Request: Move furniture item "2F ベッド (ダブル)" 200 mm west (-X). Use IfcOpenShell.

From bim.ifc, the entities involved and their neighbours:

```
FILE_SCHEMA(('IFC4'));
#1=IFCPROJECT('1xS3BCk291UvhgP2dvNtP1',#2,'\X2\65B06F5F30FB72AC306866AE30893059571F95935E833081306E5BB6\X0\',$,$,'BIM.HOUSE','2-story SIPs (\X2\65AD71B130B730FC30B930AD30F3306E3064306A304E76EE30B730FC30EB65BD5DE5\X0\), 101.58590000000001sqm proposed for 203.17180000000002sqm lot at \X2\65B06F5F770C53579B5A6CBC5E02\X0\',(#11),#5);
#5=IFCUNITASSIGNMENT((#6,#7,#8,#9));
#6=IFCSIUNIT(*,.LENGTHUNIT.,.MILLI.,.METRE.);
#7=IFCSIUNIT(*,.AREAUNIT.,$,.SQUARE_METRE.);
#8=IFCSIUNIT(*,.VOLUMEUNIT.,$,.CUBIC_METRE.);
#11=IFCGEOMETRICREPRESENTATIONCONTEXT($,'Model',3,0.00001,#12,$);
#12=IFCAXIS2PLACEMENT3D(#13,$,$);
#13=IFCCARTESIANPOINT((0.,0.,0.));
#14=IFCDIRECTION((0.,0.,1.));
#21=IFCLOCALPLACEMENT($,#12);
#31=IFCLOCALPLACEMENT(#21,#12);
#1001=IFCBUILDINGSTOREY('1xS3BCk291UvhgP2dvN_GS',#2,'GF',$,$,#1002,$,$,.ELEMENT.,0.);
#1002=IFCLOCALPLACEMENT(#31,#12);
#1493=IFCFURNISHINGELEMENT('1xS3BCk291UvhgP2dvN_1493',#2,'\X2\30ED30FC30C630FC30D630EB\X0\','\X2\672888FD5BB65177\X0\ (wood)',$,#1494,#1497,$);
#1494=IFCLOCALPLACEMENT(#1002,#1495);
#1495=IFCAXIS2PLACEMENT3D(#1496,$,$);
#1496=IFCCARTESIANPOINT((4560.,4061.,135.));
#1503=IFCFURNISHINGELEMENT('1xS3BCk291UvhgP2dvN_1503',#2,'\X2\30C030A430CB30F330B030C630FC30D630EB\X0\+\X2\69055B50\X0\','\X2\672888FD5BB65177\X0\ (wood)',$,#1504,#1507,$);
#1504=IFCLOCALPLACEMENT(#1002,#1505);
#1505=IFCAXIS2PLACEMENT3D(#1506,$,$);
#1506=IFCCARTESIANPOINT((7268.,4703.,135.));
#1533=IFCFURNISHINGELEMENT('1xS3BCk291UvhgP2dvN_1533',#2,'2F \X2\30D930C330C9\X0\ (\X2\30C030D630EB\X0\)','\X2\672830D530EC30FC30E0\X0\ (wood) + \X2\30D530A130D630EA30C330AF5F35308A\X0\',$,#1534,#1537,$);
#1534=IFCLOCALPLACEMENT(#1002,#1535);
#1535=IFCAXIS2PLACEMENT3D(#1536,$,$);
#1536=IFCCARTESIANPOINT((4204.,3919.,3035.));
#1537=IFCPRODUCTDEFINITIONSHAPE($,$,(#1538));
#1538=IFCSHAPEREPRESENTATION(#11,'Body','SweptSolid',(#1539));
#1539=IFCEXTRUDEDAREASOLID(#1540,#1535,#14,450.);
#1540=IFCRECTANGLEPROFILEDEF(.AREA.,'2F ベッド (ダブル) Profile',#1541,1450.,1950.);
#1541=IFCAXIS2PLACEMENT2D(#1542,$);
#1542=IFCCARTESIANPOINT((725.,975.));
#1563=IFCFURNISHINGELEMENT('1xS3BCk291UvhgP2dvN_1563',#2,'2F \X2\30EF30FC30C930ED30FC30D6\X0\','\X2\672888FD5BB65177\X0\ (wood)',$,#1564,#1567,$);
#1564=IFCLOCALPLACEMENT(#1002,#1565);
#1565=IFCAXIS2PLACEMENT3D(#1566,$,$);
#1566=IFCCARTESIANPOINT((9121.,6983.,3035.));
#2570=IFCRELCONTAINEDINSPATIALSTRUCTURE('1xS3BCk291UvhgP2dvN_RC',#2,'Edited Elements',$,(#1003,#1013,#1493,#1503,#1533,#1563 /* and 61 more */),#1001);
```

```python
import ifcopenshell
import ifcopenshell.api.geometry
import ifcopenshell.util.placement

model = ifcopenshell.open("bim.ifc")

item = model.by_id(1533)
matrix = ifcopenshell.util.placement.get_local_placement(item.ObjectPlacement)
matrix[0, 3] -= 200.0
ifcopenshell.api.geometry.edit_object_placement(model, product=item, matrix=matrix, is_si=False)

print(ifcopenshell.util.placement.get_local_placement(item.ObjectPlacement).round(3) + 0.0)

model.write("bim_edited.ifc")
```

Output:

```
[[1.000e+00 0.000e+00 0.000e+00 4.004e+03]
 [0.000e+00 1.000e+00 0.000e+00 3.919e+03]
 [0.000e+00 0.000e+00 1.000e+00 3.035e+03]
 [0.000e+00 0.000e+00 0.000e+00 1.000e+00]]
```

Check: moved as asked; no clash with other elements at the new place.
